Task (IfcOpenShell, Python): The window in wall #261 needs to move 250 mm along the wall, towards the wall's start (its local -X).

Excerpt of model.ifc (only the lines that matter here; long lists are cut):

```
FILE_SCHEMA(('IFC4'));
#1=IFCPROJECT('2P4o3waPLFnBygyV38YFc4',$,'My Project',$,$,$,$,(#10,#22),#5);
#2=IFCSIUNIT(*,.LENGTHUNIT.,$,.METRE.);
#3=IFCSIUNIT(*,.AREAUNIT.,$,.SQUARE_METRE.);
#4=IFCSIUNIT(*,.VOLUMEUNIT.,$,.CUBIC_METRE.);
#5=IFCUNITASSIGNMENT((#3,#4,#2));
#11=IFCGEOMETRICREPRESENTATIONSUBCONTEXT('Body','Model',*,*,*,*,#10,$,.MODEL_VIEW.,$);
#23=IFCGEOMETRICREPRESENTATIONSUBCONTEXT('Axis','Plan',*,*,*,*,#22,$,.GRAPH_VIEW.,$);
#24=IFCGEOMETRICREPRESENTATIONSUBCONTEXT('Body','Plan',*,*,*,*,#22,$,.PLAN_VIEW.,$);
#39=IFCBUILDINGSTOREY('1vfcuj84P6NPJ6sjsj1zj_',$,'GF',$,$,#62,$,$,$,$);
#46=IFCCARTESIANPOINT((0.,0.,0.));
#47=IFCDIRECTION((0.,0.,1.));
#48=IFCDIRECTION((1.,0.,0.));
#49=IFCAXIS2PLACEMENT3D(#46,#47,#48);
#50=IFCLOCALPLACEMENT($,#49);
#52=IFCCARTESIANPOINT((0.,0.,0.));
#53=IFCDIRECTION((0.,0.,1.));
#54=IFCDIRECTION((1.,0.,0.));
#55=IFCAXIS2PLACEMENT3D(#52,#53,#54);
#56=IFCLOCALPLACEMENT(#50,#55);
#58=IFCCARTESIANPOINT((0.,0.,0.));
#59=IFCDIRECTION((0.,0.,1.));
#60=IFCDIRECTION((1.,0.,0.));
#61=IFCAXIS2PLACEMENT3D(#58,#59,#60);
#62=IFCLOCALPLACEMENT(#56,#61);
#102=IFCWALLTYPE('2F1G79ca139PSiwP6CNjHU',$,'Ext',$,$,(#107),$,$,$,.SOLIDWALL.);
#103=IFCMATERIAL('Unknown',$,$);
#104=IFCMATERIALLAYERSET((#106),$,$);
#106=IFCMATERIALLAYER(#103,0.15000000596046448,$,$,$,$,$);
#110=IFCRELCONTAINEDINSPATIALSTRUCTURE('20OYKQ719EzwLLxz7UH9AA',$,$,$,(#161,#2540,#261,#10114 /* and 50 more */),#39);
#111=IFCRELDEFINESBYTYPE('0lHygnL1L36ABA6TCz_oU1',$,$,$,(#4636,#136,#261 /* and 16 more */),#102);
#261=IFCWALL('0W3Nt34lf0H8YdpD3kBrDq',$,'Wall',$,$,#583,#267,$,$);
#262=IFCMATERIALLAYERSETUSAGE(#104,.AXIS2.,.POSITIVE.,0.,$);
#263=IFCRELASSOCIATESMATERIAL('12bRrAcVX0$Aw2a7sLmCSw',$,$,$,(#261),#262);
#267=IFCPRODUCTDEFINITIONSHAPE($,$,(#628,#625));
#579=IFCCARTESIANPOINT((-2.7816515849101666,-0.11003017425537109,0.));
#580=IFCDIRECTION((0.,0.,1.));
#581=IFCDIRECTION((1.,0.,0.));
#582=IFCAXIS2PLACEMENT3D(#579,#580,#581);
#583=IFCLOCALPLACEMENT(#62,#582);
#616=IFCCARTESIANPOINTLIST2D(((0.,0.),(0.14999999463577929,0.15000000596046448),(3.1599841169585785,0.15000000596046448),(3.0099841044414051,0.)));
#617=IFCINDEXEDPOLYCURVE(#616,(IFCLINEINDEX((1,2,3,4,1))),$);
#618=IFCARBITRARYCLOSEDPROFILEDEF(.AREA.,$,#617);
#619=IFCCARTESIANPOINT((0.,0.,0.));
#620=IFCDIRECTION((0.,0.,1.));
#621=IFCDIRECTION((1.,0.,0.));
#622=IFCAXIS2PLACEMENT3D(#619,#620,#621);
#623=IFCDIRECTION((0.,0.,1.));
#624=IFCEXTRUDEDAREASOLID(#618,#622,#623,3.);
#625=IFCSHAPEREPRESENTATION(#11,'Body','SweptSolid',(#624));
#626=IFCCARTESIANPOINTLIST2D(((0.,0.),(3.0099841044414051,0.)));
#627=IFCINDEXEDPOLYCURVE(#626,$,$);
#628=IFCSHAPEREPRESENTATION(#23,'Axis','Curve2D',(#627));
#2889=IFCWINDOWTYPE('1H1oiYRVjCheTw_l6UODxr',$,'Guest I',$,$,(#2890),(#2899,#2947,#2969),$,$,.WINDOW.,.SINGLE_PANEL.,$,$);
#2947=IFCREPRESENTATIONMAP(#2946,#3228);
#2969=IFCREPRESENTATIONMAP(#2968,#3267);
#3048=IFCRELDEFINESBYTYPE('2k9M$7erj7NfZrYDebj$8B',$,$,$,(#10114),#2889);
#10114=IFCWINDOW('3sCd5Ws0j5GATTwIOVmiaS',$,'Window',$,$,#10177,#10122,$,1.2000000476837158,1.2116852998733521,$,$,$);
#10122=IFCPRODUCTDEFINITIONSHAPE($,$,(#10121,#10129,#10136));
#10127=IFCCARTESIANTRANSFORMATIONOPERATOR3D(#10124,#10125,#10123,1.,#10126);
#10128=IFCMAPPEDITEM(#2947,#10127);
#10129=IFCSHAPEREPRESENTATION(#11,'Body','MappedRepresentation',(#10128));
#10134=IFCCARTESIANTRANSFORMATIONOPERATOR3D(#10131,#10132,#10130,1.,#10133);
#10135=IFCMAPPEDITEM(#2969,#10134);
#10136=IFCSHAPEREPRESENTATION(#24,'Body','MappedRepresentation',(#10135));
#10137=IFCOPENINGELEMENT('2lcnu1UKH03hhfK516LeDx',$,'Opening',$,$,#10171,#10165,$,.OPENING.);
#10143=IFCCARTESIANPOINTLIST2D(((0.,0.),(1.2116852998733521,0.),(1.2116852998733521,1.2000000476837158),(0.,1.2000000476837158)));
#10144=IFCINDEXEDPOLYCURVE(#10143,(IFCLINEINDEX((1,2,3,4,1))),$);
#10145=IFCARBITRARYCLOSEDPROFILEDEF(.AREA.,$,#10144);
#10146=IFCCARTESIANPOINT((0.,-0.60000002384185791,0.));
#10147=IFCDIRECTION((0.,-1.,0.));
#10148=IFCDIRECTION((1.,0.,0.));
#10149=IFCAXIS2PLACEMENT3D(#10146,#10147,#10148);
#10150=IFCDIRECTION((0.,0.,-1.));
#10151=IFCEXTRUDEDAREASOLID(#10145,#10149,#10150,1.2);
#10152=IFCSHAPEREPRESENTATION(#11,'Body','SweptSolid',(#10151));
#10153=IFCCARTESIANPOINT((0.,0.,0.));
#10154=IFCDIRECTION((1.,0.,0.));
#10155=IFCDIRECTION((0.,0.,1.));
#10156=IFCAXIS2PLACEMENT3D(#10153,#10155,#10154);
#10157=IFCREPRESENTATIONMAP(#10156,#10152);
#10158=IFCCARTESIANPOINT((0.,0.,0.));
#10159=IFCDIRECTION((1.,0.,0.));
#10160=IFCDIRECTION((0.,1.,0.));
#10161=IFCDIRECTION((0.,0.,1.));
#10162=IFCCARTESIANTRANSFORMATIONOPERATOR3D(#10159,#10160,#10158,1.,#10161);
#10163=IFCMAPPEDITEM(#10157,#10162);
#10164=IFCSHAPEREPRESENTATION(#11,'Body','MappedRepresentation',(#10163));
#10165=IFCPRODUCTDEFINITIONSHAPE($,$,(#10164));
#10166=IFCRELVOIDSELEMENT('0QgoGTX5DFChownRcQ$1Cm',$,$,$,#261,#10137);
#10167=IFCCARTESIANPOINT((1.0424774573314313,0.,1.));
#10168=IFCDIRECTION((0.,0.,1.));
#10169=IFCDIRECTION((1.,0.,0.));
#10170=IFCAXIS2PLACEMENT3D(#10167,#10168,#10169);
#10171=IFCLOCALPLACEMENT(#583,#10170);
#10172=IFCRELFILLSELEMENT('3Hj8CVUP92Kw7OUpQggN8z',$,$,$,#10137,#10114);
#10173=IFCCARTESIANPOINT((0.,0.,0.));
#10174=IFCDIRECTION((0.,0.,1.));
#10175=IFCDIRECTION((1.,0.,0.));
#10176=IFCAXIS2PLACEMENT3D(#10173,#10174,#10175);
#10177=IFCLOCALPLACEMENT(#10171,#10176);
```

```python
import ifcopenshell
import ifcopenshell.api.geometry
import ifcopenshell.util.placement
import ifcopenshell.util.unit

model = ifcopenshell.open("model.ifc")
unit_scale = ifcopenshell.util.unit.calculate_unit_scale(model)

window = model.by_id(10114)
opening = window.FillsVoids[0].RelatingOpeningElement
wall = opening.VoidsElements[0].RelatingBuildingElement

wall_matrix = ifcopenshell.util.placement.get_local_placement(wall.ObjectPlacement)
shift = wall_matrix[:3, 0] * -0.25 / unit_scale
before = ifcopenshell.util.placement.get_local_placement(window.ObjectPlacement)[:3, 3].copy()

# The window is placed relative to its opening, so it follows when the opening moves.
matrix = ifcopenshell.util.placement.get_local_placement(opening.ObjectPlacement)
matrix[:3, 3] += shift
ifcopenshell.api.geometry.edit_object_placement(
    model, product=opening, matrix=matrix, is_si=False, should_transform_children=True
)

after = ifcopenshell.util.placement.get_local_placement(window.ObjectPlacement)[:3, 3]
print("window moved by", (after - before).round(3) + 0.0)

model.write("model_rev.ifc")
```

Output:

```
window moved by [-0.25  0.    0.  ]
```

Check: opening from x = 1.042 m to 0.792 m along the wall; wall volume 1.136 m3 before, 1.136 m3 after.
